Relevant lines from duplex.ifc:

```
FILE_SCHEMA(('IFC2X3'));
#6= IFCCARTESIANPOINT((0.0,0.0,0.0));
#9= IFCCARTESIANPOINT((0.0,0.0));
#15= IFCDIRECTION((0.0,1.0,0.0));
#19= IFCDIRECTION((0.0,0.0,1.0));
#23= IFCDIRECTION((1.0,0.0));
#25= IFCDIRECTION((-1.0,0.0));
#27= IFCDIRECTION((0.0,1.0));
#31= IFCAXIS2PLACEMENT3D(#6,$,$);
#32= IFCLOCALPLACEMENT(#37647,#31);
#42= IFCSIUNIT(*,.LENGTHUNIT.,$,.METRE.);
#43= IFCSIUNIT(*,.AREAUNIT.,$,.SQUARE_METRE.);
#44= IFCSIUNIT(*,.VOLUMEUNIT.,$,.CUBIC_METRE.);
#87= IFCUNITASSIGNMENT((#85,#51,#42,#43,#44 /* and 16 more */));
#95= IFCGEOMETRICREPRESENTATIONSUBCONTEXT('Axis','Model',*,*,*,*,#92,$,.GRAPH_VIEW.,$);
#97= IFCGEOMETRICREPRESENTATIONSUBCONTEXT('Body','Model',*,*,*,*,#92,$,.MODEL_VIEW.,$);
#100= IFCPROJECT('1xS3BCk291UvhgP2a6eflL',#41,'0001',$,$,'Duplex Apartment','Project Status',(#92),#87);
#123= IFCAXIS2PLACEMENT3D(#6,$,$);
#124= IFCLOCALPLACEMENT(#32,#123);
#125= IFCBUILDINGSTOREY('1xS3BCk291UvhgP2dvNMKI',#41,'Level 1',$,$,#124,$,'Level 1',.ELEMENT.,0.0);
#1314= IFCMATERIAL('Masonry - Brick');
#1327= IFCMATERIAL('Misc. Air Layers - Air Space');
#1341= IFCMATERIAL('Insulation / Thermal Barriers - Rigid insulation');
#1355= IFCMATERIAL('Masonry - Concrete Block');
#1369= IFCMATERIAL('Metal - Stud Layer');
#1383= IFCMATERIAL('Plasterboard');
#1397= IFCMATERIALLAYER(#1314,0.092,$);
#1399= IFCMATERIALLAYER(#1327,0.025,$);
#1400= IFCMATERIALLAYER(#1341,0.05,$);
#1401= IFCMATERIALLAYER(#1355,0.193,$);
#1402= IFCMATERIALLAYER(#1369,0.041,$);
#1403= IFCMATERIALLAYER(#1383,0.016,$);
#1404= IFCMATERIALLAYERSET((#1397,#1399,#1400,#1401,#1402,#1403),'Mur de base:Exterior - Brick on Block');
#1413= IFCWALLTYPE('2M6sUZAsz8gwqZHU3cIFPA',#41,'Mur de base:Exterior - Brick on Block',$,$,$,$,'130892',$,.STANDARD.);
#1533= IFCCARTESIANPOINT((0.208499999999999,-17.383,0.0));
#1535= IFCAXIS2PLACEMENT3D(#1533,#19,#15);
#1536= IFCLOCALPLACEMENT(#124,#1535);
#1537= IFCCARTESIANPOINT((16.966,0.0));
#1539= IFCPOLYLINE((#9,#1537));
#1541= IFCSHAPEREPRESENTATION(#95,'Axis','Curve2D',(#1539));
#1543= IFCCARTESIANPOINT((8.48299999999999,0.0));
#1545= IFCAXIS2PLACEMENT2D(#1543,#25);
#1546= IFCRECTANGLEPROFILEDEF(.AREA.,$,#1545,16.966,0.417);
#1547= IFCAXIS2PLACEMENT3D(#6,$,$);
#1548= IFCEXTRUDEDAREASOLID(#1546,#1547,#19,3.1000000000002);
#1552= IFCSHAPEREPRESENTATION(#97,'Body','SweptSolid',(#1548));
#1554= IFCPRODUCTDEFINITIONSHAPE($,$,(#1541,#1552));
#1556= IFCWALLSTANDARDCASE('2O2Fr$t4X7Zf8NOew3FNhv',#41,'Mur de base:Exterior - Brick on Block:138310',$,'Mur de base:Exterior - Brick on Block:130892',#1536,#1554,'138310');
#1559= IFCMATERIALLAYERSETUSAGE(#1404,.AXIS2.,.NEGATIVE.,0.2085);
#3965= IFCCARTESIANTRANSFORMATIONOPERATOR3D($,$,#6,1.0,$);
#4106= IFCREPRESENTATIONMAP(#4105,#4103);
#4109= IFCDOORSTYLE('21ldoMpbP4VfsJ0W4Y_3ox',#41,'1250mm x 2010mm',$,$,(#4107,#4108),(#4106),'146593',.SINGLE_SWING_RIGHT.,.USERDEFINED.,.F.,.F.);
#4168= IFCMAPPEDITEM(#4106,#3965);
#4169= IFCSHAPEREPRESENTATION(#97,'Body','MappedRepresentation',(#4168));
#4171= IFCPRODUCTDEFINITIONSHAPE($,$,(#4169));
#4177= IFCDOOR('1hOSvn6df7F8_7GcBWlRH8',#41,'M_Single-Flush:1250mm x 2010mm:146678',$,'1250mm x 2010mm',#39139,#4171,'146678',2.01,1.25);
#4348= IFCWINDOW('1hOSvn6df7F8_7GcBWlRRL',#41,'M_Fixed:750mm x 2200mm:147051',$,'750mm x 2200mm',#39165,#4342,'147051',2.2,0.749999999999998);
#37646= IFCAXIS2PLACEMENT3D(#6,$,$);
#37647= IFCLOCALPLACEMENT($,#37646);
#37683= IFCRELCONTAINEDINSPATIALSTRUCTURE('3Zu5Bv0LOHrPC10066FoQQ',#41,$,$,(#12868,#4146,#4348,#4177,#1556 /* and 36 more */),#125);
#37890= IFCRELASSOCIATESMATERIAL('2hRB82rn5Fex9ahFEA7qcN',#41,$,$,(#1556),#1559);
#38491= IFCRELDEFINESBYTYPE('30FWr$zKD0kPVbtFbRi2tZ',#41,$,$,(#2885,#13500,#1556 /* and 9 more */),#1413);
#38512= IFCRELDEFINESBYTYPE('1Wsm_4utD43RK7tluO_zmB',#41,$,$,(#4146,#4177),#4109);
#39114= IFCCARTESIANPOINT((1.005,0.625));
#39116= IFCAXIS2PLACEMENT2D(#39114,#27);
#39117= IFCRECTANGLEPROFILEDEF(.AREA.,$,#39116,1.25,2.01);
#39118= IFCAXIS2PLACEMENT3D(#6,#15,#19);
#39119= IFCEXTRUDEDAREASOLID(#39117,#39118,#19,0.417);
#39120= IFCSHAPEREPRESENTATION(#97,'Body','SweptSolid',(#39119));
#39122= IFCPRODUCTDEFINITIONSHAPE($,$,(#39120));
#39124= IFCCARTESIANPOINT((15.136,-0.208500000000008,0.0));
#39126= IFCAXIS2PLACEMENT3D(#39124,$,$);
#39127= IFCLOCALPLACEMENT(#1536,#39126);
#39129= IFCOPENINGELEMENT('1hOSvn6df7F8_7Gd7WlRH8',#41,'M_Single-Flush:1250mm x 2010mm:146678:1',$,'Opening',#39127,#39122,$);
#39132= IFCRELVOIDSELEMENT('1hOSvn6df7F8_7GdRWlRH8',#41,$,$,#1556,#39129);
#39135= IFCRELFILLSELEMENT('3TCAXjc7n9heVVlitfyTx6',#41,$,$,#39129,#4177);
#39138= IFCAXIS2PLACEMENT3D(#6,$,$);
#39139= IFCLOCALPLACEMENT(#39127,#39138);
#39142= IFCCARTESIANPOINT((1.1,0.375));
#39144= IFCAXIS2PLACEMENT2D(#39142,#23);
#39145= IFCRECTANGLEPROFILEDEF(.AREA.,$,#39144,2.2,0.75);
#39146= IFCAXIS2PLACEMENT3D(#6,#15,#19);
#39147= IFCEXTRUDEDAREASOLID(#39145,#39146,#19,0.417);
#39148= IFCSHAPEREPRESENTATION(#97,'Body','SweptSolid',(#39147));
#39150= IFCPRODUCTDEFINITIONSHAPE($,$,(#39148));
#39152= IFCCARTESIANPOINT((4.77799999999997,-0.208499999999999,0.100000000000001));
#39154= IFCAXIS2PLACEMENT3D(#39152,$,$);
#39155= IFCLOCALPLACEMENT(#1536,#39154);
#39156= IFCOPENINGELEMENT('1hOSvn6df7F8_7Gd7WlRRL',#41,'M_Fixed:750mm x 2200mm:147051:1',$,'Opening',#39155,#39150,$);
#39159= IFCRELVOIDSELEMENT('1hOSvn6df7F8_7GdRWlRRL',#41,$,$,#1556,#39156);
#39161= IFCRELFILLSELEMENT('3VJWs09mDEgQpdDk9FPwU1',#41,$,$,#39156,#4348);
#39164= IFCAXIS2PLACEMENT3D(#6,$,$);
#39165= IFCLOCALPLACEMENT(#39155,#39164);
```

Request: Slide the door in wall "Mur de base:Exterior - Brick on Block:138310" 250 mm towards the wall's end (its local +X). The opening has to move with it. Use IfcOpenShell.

```python
import ifcopenshell
import ifcopenshell.api.geometry
import ifcopenshell.util.placement
import ifcopenshell.util.unit

model = ifcopenshell.open("duplex.ifc")
unit_scale = ifcopenshell.util.unit.calculate_unit_scale(model)

door = model.by_id(4177)
opening = door.FillsVoids[0].RelatingOpeningElement
wall = opening.VoidsElements[0].RelatingBuildingElement

wall_matrix = ifcopenshell.util.placement.get_local_placement(wall.ObjectPlacement)
shift = wall_matrix[:3, 0] * 0.25 / unit_scale
before = ifcopenshell.util.placement.get_local_placement(door.ObjectPlacement)[:3, 3].copy()

# The door is placed relative to its opening, so it follows when the opening moves.
matrix = ifcopenshell.util.placement.get_local_placement(opening.ObjectPlacement)
matrix[:3, 3] += shift
ifcopenshell.api.geometry.edit_object_placement(
    model, product=opening, matrix=matrix, is_si=False, should_transform_children=True
)

after = ifcopenshell.util.placement.get_local_placement(door.ObjectPlacement)[:3, 3]
print("door moved by", (after - before).round(3) + 0.0)

model.write("duplex_edited.ifc")
```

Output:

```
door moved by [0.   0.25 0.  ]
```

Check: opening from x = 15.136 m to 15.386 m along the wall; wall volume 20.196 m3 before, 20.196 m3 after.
